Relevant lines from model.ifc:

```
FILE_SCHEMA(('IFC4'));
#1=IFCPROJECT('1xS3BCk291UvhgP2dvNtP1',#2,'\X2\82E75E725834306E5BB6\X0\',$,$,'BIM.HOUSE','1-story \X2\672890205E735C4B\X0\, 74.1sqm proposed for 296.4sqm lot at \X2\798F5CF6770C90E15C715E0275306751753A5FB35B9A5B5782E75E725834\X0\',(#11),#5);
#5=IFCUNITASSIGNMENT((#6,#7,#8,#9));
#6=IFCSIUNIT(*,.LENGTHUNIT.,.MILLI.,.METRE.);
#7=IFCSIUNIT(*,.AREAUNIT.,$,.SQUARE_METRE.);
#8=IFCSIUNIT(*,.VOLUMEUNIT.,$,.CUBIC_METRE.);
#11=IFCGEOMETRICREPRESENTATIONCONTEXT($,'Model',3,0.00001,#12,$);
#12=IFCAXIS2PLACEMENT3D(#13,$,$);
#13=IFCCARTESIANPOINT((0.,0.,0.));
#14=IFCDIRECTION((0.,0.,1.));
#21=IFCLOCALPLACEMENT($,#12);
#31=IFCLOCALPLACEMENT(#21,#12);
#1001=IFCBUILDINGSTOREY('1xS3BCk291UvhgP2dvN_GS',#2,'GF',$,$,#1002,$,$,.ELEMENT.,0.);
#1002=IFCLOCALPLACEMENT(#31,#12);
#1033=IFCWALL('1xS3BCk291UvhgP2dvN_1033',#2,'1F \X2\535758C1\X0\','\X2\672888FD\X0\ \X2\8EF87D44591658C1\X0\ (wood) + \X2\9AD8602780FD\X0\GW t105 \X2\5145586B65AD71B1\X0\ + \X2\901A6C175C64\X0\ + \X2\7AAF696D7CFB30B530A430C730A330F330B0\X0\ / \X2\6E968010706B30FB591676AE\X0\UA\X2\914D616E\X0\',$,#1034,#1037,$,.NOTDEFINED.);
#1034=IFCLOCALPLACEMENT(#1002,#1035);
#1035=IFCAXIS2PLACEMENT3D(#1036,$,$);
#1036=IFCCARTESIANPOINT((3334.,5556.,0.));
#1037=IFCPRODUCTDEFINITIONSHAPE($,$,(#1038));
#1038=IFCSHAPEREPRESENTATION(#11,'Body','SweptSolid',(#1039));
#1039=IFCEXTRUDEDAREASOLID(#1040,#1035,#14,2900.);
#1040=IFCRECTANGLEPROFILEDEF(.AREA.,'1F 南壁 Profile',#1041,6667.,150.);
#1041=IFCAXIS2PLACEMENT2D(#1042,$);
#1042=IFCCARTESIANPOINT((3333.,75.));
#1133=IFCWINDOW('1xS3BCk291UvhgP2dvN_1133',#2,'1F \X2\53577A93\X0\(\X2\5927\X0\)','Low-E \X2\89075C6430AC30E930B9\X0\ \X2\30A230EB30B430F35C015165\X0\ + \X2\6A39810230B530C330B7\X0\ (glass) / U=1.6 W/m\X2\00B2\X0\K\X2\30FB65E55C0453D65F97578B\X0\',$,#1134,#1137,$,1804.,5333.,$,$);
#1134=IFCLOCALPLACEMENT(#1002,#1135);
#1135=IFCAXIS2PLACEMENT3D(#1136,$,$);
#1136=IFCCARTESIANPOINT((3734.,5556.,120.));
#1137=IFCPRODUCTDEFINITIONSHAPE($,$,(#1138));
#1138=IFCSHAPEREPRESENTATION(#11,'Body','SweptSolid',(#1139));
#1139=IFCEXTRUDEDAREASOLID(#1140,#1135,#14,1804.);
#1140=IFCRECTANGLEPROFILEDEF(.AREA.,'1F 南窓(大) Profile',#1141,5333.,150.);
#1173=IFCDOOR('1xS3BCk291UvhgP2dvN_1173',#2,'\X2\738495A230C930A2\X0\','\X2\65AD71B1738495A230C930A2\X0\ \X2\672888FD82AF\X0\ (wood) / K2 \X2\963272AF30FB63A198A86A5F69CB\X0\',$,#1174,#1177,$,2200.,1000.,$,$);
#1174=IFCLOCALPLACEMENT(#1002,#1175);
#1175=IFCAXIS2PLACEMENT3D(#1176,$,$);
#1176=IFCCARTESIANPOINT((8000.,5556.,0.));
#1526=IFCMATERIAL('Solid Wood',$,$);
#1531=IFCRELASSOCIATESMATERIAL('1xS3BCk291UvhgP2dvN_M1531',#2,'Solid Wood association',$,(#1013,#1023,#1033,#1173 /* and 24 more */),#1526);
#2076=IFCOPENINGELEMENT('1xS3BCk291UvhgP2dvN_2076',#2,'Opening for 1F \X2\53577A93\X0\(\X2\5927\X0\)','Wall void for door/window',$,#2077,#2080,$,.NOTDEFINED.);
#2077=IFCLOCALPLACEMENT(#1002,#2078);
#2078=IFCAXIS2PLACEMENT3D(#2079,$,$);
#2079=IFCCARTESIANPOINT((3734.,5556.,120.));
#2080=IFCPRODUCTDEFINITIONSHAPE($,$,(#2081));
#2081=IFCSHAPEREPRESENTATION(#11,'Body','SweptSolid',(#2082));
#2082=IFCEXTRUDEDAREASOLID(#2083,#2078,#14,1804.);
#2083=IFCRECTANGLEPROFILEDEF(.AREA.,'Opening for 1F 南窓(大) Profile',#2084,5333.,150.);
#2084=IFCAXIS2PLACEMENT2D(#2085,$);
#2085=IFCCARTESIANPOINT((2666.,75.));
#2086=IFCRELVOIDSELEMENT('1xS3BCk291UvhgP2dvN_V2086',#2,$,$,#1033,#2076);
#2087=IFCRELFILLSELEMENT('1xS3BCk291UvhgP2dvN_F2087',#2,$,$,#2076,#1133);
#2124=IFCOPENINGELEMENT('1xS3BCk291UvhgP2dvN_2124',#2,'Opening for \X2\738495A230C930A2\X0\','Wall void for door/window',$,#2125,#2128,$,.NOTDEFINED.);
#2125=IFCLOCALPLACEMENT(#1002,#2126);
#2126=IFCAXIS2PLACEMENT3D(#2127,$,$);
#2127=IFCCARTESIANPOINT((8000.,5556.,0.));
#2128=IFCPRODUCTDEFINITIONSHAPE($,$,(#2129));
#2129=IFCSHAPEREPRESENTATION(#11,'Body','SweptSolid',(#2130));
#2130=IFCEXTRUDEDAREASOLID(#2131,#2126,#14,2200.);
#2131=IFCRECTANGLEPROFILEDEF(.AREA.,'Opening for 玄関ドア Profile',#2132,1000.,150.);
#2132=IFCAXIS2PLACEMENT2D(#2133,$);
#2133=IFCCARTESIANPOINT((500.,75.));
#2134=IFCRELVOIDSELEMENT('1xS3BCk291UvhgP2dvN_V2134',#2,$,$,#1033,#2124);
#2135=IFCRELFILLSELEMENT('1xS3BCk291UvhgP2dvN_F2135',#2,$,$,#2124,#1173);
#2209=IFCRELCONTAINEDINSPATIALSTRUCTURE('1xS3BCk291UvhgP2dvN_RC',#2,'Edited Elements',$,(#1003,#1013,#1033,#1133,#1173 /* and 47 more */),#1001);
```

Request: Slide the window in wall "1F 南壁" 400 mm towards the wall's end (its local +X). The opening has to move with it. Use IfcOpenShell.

```python
import ifcopenshell
import ifcopenshell.api.geometry
import ifcopenshell.util.placement
import ifcopenshell.util.unit

model = ifcopenshell.open("model.ifc")
unit_scale = ifcopenshell.util.unit.calculate_unit_scale(model)

window = model.by_guid("1xS3BCk291UvhgP2dvN_1133")
opening = window.FillsVoids[0].RelatingOpeningElement
wall = opening.VoidsElements[0].RelatingBuildingElement

wall_matrix = ifcopenshell.util.placement.get_local_placement(wall.ObjectPlacement)
shift = wall_matrix[:3, 0] * 0.4 / unit_scale
before = ifcopenshell.util.placement.get_local_placement(window.ObjectPlacement)[:3, 3].copy()

# The window is not placed relative to its opening, so move both.
for product in (opening, window):
    matrix = ifcopenshell.util.placement.get_local_placement(product.ObjectPlacement)
    matrix[:3, 3] += shift
    ifcopenshell.api.geometry.edit_object_placement(model, product=product, matrix=matrix, is_si=False)

after = ifcopenshell.util.placement.get_local_placement(window.ObjectPlacement)[:3, 3]
print("window moved by", (after - before).round(3) + 0.0)

model.write("model_edited.ifc")
```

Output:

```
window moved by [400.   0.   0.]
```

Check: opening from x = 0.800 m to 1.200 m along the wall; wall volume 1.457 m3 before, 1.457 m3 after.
